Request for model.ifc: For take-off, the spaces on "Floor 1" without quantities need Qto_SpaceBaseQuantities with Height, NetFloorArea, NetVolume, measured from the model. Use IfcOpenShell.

First a look at what the model holds.

```python
import ifcopenshell
import ifcopenshell.util.element
import ifcopenshell.util.unit

model = ifcopenshell.open("model.ifc")
print(model.schema)
for unit_type in ("LENGTHUNIT", "AREAUNIT", "VOLUMEUNIT"):
    print(unit_type, ifcopenshell.util.unit.calculate_unit_scale(model, unit_type))
storey = next(s for s in model.by_type("IfcBuildingStorey") if s.Name == "Floor 1")
spaces = [e for e in ifcopenshell.util.element.get_decomposition(storey) if e.is_a("IfcSpace")]
for e in sorted(spaces, key=lambda e: e.id()):
    print(e.id(), e.is_a(), e.Name, list(ifcopenshell.util.element.get_psets(e, qtos_only=True)), sep=" | ")
```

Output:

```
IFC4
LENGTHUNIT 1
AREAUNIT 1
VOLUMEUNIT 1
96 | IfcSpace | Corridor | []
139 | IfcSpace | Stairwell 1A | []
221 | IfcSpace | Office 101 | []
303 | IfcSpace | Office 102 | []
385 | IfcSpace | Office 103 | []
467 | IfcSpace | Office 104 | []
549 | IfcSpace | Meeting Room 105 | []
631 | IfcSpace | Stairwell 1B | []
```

```python
import ifcopenshell
import ifcopenshell.api.pset
import ifcopenshell.geom
import ifcopenshell.util.element
import ifcopenshell.util.shape
import ifcopenshell.util.unit

model = ifcopenshell.open("model.ifc")
unit_scale = ifcopenshell.util.unit.calculate_unit_scale(model)
area_scale = ifcopenshell.util.unit.calculate_unit_scale(model, "AREAUNIT")
volume_scale = ifcopenshell.util.unit.calculate_unit_scale(model, "VOLUMEUNIT")
settings = ifcopenshell.geom.settings()

storey = next(s for s in model.by_type("IfcBuildingStorey") if s.Name == "Floor 1")
spaces = [e for e in ifcopenshell.util.element.get_decomposition(storey) if e.is_a("IfcSpace")]

for e in sorted(spaces, key=lambda e: e.id()):
    if ifcopenshell.util.element.get_psets(e, qtos_only=True, should_inherit=False):
        continue
    # Geometry comes back in metres, in the element's own axes.
    shape = ifcopenshell.geom.create_shape(settings, e)
    values = {
        "Height": ifcopenshell.util.shape.get_z(shape.geometry) / unit_scale,
        "NetFloorArea": ifcopenshell.util.shape.get_footprint_area(shape.geometry) / area_scale,
        "NetVolume": ifcopenshell.util.shape.get_volume(shape.geometry) / volume_scale,
    }
    qto = ifcopenshell.api.pset.add_qto(model, product=e, name="Qto_SpaceBaseQuantities")
    ifcopenshell.api.pset.edit_qto(model, qto=qto, properties=values)
    print(e.id(), {k: round(v, 3) for k, v in values.items()})

model.write("model_v2.ifc")
```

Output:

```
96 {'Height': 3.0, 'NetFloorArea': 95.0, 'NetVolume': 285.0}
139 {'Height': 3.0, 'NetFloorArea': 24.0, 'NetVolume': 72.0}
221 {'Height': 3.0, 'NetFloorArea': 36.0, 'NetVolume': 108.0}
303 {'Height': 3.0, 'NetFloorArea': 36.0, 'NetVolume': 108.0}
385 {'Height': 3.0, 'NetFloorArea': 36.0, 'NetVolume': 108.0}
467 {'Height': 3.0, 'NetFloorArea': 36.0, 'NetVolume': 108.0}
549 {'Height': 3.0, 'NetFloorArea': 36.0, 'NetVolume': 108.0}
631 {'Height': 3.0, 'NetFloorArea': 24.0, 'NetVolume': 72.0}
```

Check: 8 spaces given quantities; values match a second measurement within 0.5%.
